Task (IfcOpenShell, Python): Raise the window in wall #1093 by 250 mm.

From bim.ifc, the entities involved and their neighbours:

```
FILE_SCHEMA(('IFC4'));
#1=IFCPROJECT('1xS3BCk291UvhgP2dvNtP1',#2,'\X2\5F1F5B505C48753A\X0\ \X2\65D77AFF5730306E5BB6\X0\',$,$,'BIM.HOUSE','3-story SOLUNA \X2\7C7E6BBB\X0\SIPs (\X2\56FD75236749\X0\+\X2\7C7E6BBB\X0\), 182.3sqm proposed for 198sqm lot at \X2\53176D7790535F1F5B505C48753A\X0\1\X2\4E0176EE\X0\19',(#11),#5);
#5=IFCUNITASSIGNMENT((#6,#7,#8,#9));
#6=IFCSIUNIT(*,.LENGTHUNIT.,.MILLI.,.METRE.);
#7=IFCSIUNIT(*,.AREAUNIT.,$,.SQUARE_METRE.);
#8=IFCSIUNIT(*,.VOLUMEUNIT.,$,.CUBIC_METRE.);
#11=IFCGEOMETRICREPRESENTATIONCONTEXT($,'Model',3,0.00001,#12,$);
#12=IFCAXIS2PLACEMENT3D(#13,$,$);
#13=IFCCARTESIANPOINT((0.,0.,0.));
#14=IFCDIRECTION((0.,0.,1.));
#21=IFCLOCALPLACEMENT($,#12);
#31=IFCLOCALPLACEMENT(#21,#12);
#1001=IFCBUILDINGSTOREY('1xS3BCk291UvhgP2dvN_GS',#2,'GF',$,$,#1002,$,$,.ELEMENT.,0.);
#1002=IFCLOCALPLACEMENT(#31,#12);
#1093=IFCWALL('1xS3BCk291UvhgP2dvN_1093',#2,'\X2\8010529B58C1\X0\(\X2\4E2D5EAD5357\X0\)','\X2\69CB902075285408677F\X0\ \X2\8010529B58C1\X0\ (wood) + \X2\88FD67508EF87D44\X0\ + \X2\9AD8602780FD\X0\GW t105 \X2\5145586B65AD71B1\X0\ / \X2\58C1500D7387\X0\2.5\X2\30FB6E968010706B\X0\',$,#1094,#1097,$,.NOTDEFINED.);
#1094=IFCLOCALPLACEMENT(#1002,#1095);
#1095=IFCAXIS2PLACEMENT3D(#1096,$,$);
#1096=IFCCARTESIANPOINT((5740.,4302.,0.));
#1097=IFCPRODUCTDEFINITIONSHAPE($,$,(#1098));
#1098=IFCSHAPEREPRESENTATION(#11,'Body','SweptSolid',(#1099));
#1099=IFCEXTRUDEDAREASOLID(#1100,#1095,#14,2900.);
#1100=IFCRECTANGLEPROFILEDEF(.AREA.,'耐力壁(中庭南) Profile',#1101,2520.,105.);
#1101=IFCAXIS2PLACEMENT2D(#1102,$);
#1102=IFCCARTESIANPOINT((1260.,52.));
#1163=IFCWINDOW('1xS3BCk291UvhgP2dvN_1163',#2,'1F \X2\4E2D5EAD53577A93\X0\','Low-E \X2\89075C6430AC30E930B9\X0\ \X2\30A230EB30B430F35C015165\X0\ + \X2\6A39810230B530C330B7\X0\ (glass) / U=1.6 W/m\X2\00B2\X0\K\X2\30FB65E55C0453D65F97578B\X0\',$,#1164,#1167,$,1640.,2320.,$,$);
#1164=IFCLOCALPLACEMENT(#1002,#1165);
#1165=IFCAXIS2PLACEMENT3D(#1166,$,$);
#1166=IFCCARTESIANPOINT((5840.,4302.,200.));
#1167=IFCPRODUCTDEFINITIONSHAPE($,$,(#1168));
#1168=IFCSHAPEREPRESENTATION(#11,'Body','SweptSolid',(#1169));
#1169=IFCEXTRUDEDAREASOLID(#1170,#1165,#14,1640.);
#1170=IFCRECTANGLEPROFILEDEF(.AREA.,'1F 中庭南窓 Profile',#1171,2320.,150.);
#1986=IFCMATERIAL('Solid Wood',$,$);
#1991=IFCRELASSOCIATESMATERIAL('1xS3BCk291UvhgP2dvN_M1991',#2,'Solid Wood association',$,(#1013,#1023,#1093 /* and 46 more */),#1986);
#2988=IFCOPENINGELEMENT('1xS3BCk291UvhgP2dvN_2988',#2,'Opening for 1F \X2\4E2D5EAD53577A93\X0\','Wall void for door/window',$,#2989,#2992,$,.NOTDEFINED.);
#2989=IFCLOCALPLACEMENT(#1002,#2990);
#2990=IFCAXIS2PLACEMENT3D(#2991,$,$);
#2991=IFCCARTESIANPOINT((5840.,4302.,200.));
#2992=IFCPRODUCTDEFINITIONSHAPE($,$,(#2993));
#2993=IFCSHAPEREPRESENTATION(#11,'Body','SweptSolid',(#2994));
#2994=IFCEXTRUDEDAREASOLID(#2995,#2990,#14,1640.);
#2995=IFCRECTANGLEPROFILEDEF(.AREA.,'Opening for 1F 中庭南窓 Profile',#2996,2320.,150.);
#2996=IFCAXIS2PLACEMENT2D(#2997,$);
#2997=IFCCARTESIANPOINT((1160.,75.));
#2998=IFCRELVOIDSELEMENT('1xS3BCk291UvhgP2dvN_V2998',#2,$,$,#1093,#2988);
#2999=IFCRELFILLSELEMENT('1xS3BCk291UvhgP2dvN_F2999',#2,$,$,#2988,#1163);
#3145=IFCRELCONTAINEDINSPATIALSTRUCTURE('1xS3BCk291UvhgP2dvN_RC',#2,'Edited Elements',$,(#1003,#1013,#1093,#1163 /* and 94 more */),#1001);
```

```python
import numpy as np
import ifcopenshell
import ifcopenshell.api.geometry
import ifcopenshell.util.placement
import ifcopenshell.util.unit

model = ifcopenshell.open("bim.ifc")
unit_scale = ifcopenshell.util.unit.calculate_unit_scale(model)

window = model.by_guid("1xS3BCk291UvhgP2dvN_1163")
opening = window.FillsVoids[0].RelatingOpeningElement
dz = 0.25 / unit_scale

shift = np.array([0.0, 0.0, dz])
# The window is not placed relative to its opening, so move both.
for product in (opening, window):
    matrix = ifcopenshell.util.placement.get_local_placement(product.ObjectPlacement)
    matrix[:3, 3] += shift
    ifcopenshell.api.geometry.edit_object_placement(model, product=product, matrix=matrix, is_si=False)

print(f"moved by {dz * unit_scale:+.3f} m")

model.write("bim_updated.ifc")
```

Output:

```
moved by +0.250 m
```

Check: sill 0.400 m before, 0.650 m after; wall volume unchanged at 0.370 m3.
